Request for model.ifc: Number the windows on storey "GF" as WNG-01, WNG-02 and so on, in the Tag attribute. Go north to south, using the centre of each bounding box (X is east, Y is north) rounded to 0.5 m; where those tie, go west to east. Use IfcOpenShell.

First a look at what the model holds.

```python
import ifcopenshell
import ifcopenshell.util.element
import ifcopenshell.util.placement

model = ifcopenshell.open("model.ifc")
print(model.schema)
storey = next(s for s in model.by_type("IfcBuildingStorey") if s.Name == "GF")
windows = [e for e in ifcopenshell.util.element.get_decomposition(storey) if e.is_a("IfcWindow")]
for e in sorted(windows, key=lambda e: e.id()):
    origin = ifcopenshell.util.placement.get_local_placement(e.ObjectPlacement)[:3, 3]
    print(e.id(), e.Tag, e.Name, origin.round(2) + 0.0, sep=" | ")
```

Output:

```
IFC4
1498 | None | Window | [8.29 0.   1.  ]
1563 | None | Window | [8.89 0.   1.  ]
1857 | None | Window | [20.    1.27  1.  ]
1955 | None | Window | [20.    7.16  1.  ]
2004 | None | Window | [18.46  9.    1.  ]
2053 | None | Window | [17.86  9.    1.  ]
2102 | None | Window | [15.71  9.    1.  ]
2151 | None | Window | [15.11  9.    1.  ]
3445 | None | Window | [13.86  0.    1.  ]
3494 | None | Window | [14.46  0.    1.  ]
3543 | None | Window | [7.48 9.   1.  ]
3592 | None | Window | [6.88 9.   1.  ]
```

```python
import ifcopenshell
import ifcopenshell.geom
import ifcopenshell.util.element
import ifcopenshell.util.shape

model = ifcopenshell.open("model.ifc")
settings = ifcopenshell.geom.settings()
settings.set("use-world-coords", True)


def centre(element):
    shape = ifcopenshell.geom.create_shape(settings, element)
    return ifcopenshell.util.shape.get_bbox_centroid(shape.geometry)


storey = next(s for s in model.by_type("IfcBuildingStorey") if s.Name == "GF")
windows = [e for e in ifcopenshell.util.element.get_decomposition(storey) if e.is_a("IfcWindow")]

# Insertion points can sit at a corner or the storey origin, so sort by the geometry (in metres).
centres = {e: centre(e) for e in windows}
windows.sort(key=lambda e: (-round(centres[e][1] / 0.5), centres[e][0]))

for i, e in enumerate(windows, start=1):
    number = f"WNG-{i:02d}"
    e.Tag = number
    print(e.id(), number)

model.write("model_edited.ifc")
```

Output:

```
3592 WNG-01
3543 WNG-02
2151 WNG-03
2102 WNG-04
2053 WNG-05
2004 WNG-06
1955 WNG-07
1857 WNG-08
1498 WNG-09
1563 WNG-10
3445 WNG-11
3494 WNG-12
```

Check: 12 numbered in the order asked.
